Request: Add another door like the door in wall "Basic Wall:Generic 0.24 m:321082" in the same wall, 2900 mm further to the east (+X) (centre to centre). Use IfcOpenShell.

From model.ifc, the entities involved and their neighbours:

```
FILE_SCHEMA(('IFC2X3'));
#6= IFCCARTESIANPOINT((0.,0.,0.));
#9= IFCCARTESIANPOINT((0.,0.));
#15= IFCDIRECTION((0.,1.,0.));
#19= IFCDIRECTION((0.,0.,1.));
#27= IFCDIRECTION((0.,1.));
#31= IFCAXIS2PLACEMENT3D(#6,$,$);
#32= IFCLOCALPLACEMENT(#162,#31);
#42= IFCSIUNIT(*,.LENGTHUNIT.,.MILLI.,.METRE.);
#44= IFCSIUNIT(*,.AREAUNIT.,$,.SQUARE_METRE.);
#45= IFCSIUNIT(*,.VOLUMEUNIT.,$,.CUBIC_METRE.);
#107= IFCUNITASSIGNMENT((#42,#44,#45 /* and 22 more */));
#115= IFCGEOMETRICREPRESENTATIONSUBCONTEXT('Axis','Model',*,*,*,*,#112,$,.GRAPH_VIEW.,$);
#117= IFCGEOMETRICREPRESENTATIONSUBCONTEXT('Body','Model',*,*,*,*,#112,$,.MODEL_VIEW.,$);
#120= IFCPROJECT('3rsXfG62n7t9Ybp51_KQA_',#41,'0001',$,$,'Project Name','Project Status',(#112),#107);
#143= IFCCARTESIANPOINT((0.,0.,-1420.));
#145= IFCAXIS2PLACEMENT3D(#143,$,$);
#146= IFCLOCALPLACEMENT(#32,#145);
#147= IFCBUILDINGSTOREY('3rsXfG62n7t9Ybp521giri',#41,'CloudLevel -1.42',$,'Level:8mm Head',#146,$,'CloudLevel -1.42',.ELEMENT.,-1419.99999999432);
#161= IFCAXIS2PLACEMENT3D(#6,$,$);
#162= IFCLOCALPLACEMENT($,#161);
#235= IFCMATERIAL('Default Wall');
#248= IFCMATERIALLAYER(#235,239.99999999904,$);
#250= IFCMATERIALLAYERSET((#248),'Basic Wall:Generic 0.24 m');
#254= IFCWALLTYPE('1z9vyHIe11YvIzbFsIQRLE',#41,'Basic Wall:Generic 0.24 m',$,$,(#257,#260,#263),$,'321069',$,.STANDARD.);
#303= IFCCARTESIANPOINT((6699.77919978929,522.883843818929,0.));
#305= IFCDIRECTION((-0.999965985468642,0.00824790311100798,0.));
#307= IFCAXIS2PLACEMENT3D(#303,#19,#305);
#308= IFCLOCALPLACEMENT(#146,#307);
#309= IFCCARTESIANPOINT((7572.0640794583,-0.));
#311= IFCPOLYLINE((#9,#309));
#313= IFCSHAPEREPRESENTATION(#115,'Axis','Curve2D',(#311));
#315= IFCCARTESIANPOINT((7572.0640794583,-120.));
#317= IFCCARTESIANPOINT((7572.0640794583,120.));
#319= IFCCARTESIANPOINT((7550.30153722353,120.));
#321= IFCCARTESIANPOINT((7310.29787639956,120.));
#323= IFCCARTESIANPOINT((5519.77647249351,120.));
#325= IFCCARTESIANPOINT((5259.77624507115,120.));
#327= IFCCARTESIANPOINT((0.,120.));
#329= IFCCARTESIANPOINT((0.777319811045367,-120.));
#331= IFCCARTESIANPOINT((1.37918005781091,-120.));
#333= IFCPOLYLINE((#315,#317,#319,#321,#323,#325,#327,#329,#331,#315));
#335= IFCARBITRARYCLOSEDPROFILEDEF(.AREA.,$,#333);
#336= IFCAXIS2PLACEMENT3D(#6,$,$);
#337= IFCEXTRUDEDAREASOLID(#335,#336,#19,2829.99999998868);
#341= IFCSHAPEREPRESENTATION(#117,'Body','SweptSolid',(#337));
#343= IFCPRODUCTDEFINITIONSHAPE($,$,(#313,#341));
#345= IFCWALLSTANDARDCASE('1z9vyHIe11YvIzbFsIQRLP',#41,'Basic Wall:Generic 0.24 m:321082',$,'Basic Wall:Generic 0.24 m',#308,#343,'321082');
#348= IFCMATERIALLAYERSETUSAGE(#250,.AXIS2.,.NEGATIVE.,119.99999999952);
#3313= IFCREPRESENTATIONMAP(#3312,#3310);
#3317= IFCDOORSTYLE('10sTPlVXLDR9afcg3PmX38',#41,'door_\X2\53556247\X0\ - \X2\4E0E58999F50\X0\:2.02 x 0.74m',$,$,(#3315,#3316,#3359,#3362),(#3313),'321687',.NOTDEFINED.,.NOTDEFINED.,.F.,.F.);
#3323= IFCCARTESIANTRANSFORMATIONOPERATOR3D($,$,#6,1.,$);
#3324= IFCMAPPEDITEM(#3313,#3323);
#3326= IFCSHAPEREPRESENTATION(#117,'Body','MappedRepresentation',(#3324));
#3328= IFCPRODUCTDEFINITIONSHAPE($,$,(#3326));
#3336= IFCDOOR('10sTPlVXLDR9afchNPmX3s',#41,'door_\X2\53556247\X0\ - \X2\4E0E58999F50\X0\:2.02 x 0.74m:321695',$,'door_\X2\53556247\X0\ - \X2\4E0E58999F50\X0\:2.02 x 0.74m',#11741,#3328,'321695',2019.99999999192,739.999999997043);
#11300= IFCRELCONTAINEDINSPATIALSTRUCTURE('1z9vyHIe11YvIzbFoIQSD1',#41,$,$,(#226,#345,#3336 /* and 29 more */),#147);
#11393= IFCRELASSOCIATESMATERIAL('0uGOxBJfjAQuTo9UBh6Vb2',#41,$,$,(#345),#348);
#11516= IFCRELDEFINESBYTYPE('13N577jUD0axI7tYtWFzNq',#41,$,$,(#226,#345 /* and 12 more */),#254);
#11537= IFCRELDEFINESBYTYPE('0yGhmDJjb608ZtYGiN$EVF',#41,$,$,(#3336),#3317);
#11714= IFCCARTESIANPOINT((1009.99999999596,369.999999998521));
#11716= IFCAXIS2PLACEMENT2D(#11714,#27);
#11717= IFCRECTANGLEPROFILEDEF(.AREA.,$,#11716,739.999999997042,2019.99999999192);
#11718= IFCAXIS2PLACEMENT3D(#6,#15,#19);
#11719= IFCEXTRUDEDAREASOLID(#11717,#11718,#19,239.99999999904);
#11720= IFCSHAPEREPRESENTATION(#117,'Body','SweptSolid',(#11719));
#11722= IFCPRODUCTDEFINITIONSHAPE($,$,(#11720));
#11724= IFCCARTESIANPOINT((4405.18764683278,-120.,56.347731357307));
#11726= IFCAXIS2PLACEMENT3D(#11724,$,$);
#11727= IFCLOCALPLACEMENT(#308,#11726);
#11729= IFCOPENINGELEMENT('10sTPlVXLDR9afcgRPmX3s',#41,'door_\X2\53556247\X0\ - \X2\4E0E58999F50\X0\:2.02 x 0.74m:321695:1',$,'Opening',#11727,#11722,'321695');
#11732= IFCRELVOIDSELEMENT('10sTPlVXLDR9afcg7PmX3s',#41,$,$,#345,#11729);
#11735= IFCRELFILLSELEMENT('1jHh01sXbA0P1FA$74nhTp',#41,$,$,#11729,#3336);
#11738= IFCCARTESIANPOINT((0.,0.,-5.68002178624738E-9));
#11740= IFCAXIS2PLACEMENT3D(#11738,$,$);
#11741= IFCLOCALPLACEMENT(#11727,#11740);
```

```python
import ifcopenshell
import ifcopenshell.api.feature
import ifcopenshell.api.geometry
import ifcopenshell.api.root
import ifcopenshell.geom
import ifcopenshell.util.element
import ifcopenshell.util.placement
import ifcopenshell.util.shape
import ifcopenshell.util.unit

model = ifcopenshell.open("model.ifc")
unit_scale = ifcopenshell.util.unit.calculate_unit_scale(model)
settings = ifcopenshell.geom.settings()


def volume(element):
    """Net volume in cubic metres, openings subtracted."""
    shape = ifcopenshell.geom.create_shape(settings, element)
    return ifcopenshell.util.shape.get_volume(shape.geometry)


def reuse_history(source, copy):
    """copy_class also copies each property set's owner history, people and application; keep the originals."""
    for rel in copy.IsDefinedBy:
        if rel.is_a("IfcRelDefinesByProperties") and (history := rel.RelatingPropertyDefinition.OwnerHistory):
            rel.RelatingPropertyDefinition.OwnerHistory = source.OwnerHistory
            ifcopenshell.util.element.remove_deep2(model, history)


door = model.by_id(3336)
opening = door.FillsVoids[0].RelatingOpeningElement
wall = opening.VoidsElements[0].RelatingBuildingElement
before = volume(wall)
shift = ifcopenshell.util.placement.get_local_placement(wall.ObjectPlacement)[:3, 0] * -2.9 / unit_scale

# copy_class copies the void relationship, type, container and properties, but no geometry.
new_opening = ifcopenshell.api.root.copy_class(model, product=opening)
new_opening.Representation = ifcopenshell.util.element.copy_deep(
    model, opening.Representation, exclude=["IfcGeometricRepresentationContext", "IfcRepresentationMap"]
)
new_opening.Name = "door_单扇 - 与墙齐:2.02 x 0.74m"
new_opening.Tag = None
new_door = ifcopenshell.api.root.copy_class(model, product=door)
new_door.Representation = ifcopenshell.util.element.copy_deep(
    model, door.Representation, exclude=["IfcGeometricRepresentationContext", "IfcRepresentationMap"]
)
new_door.Name = "door_单扇 - 与墙齐:2.02 x 0.74m"
new_door.Tag = None
reuse_history(door, new_door)
fills = ifcopenshell.api.feature.add_filling(model, opening=new_opening, element=new_door)
fills.OwnerHistory = new_door.OwnerHistory  # required in IFC2X3

for old, new in ((opening, new_opening), (door, new_door)):
    matrix = ifcopenshell.util.placement.get_local_placement(old.ObjectPlacement)
    matrix[:3, 3] += shift
    ifcopenshell.api.geometry.edit_object_placement(model, product=new, matrix=matrix, is_si=False)

after = volume(wall)

print(f"wall volume {before:.3f} -> {after:.3f} m3")

model.write("model_edited.ifc")
```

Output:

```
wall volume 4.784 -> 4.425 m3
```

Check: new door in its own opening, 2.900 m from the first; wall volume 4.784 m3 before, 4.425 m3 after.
